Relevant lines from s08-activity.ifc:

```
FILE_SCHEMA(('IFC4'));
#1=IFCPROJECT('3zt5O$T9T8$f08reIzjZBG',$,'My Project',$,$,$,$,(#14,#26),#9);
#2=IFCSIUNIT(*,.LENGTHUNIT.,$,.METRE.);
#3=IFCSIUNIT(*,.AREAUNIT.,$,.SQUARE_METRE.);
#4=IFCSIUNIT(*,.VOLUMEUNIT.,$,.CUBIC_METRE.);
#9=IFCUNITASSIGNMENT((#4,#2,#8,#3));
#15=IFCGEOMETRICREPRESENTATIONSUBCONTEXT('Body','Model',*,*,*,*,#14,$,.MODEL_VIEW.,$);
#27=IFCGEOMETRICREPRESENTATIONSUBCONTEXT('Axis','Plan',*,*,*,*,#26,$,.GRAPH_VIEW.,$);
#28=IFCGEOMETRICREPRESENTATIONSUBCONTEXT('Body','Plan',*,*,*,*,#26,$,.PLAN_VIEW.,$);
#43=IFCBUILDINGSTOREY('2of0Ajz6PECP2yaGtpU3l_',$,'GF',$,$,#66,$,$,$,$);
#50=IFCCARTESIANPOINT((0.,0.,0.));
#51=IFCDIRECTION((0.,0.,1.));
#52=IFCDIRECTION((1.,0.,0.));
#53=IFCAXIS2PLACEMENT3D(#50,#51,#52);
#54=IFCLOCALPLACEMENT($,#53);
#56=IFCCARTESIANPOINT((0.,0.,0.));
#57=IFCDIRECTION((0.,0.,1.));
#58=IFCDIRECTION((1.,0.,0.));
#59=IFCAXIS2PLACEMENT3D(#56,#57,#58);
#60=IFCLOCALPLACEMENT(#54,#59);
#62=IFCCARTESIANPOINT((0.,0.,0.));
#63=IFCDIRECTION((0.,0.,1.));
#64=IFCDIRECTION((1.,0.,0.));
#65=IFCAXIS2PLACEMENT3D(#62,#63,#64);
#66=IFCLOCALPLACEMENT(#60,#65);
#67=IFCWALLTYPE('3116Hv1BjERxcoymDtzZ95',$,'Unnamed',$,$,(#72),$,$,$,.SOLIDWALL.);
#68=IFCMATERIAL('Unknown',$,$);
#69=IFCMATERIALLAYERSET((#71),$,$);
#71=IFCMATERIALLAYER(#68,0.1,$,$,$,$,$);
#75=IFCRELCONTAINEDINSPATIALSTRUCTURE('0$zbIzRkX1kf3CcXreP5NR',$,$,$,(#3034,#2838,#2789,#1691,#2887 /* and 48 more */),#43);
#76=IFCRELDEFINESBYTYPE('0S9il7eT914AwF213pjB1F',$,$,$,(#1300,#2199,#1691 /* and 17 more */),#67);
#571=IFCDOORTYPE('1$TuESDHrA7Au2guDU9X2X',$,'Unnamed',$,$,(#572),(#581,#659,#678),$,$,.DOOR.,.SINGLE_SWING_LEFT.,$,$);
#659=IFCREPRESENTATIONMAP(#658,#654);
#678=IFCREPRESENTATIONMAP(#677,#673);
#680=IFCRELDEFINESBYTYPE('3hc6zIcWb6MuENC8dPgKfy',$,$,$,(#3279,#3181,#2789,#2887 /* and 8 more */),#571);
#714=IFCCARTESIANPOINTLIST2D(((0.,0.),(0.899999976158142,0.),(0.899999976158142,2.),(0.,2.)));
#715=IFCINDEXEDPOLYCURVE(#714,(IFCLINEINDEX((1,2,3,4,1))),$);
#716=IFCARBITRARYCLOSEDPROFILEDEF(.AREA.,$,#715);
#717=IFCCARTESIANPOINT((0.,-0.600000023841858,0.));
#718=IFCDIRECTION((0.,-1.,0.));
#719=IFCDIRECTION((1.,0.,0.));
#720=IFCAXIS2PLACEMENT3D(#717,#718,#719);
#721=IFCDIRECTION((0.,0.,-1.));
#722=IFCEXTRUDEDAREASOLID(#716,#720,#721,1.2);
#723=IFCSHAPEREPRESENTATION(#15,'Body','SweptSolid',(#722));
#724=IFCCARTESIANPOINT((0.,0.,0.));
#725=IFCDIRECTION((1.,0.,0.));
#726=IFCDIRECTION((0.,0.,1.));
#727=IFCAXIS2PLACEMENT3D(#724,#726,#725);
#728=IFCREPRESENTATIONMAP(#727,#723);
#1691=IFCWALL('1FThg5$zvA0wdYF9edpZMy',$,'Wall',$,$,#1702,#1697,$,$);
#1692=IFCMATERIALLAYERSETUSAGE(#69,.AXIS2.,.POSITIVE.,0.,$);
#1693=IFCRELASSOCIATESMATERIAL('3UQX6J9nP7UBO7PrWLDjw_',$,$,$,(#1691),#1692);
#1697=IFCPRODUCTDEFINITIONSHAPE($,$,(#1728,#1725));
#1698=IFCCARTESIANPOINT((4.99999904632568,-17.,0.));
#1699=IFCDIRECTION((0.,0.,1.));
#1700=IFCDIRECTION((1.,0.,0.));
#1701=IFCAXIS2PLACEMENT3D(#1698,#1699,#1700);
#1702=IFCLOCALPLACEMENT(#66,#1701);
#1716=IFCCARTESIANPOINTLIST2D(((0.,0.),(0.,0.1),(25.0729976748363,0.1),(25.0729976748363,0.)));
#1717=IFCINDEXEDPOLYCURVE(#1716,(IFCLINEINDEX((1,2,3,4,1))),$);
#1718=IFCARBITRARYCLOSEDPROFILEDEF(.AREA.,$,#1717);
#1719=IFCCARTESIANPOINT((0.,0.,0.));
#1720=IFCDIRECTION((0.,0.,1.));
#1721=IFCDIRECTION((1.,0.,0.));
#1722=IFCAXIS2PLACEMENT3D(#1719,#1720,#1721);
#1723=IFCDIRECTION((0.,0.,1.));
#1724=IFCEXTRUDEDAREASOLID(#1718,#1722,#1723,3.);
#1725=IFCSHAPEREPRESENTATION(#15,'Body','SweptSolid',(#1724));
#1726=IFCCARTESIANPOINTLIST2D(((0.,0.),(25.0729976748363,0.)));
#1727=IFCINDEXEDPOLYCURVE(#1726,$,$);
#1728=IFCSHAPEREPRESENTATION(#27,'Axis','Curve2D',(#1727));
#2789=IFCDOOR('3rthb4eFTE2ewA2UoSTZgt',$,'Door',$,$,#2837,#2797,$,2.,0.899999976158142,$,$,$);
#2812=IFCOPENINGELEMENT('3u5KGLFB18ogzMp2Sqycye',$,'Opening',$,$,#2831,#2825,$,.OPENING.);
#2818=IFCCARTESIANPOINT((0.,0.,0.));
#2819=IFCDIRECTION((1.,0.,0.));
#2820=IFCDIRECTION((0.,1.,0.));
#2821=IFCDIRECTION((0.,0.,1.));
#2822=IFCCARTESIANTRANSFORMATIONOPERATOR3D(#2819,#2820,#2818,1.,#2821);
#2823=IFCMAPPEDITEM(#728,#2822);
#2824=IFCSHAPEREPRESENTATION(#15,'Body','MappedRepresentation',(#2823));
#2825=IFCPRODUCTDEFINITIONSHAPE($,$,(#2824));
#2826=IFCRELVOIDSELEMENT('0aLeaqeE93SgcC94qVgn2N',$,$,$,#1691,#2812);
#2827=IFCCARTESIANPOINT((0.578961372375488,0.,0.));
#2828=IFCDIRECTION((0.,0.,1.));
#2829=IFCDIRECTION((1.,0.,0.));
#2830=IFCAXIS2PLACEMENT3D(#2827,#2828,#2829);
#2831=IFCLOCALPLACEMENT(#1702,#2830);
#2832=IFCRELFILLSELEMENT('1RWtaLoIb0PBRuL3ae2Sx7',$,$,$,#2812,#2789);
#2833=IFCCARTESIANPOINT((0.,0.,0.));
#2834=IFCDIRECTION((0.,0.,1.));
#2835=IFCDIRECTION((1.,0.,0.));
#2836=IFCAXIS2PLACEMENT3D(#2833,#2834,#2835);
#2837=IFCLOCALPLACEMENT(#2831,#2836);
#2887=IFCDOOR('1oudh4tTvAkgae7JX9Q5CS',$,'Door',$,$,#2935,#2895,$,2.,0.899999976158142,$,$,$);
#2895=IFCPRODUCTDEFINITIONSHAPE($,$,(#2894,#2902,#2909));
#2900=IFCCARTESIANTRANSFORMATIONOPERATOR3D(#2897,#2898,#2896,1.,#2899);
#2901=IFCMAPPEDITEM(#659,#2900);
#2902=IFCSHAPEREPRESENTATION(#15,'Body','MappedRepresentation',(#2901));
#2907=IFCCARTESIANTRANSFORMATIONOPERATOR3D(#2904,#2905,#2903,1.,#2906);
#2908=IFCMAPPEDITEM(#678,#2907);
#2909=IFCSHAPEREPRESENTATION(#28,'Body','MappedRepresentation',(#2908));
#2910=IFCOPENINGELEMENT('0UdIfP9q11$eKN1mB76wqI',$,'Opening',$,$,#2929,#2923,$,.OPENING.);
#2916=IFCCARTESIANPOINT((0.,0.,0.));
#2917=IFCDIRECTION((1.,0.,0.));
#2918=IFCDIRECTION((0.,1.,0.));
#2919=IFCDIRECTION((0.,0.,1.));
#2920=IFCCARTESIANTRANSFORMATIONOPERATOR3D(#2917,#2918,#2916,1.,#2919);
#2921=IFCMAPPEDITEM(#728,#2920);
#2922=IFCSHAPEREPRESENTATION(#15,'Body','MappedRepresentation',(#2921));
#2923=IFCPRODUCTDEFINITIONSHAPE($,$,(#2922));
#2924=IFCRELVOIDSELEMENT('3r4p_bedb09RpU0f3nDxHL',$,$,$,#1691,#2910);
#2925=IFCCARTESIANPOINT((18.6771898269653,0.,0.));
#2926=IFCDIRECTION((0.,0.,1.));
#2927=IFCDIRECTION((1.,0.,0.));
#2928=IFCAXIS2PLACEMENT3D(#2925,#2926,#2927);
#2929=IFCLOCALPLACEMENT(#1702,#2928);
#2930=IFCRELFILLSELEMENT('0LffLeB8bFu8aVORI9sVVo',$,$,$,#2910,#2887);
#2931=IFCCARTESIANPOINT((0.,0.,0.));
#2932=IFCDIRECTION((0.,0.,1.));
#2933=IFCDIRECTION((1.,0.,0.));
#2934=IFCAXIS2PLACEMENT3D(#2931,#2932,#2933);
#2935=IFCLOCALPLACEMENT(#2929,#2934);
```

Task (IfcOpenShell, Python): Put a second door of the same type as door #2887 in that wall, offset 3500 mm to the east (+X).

```python
import ifcopenshell
import ifcopenshell.api.feature
import ifcopenshell.api.geometry
import ifcopenshell.api.root
import ifcopenshell.geom
import ifcopenshell.util.element
import ifcopenshell.util.placement
import ifcopenshell.util.shape
import ifcopenshell.util.unit

model = ifcopenshell.open("s08-activity.ifc")
unit_scale = ifcopenshell.util.unit.calculate_unit_scale(model)
settings = ifcopenshell.geom.settings()


def volume(element):
    """Net volume in cubic metres, openings subtracted."""
    shape = ifcopenshell.geom.create_shape(settings, element)
    return ifcopenshell.util.shape.get_volume(shape.geometry)


door = model.by_guid("1oudh4tTvAkgae7JX9Q5CS")
opening = door.FillsVoids[0].RelatingOpeningElement
wall = opening.VoidsElements[0].RelatingBuildingElement
before = volume(wall)
shift = ifcopenshell.util.placement.get_local_placement(wall.ObjectPlacement)[:3, 0] * 3.5 / unit_scale

# copy_class copies the void relationship, type, container and properties, but no geometry.
new_opening = ifcopenshell.api.root.copy_class(model, product=opening)
new_opening.Representation = ifcopenshell.util.element.copy_deep(
    model, opening.Representation, exclude=["IfcGeometricRepresentationContext", "IfcRepresentationMap"]
)
new_door = ifcopenshell.api.root.copy_class(model, product=door)
new_door.Representation = ifcopenshell.util.element.copy_deep(
    model, door.Representation, exclude=["IfcGeometricRepresentationContext", "IfcRepresentationMap"]
)
ifcopenshell.api.feature.add_filling(model, opening=new_opening, element=new_door)

for old, new in ((opening, new_opening), (door, new_door)):
    matrix = ifcopenshell.util.placement.get_local_placement(old.ObjectPlacement)
    matrix[:3, 3] += shift
    ifcopenshell.api.geometry.edit_object_placement(model, product=new, matrix=matrix, is_si=False)

after = volume(wall)

print(f"wall volume {before:.3f} -> {after:.3f} m3")

model.write("s08-activity_updated.ifc")
```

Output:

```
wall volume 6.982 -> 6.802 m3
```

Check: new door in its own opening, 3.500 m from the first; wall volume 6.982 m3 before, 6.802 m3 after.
